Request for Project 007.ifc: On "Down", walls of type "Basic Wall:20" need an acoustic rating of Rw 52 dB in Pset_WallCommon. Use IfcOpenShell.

First a look at what the model holds.

```python
import ifcopenshell
import ifcopenshell.util.element

model = ifcopenshell.open("Project 007.ifc")
print(model.schema)
storey = next(s for s in model.by_type("IfcBuildingStorey") if s.Name == "Down")
walls = [e for e in ifcopenshell.util.element.get_decomposition(storey) if e.is_a("IfcWall")]
seen = {}
for e in walls:
    element_type = ifcopenshell.util.element.get_type(e)
    key = (element_type.Name if element_type != e and element_type else None, ifcopenshell.util.element.get_pset(e, "Pset_WallCommon", "AcousticRating"))
    seen[key] = seen.get(key, 0) + 1
for (name, value), count in sorted(seen.items(), key=str):
    print(count, "x", name, "|", value)
```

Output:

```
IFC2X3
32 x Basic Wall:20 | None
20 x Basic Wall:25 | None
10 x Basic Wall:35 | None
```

```python
import ifcopenshell
import ifcopenshell.api.pset
import ifcopenshell.util.element

model = ifcopenshell.open("Project 007.ifc")

storey = next(s for s in model.by_type("IfcBuildingStorey") if s.Name == "Down")
walls = [e for e in ifcopenshell.util.element.get_decomposition(storey) if e.is_a("IfcWall")]

count = 0
for e in walls:
    element_type = ifcopenshell.util.element.get_type(e)
    if element_type in (None, e) or element_type.Name != "Basic Wall:20":
        continue
    # add_pset returns the element's existing set when there is one.
    pset = ifcopenshell.api.pset.add_pset(model, product=e, name="Pset_WallCommon")
    ifcopenshell.api.pset.edit_pset(model, pset=pset, properties={"AcousticRating": "Rw 52 dB"})
    count += 1

print(count, "walls updated")

model.write("Project 007_v2.ifc")
```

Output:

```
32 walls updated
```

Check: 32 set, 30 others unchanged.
